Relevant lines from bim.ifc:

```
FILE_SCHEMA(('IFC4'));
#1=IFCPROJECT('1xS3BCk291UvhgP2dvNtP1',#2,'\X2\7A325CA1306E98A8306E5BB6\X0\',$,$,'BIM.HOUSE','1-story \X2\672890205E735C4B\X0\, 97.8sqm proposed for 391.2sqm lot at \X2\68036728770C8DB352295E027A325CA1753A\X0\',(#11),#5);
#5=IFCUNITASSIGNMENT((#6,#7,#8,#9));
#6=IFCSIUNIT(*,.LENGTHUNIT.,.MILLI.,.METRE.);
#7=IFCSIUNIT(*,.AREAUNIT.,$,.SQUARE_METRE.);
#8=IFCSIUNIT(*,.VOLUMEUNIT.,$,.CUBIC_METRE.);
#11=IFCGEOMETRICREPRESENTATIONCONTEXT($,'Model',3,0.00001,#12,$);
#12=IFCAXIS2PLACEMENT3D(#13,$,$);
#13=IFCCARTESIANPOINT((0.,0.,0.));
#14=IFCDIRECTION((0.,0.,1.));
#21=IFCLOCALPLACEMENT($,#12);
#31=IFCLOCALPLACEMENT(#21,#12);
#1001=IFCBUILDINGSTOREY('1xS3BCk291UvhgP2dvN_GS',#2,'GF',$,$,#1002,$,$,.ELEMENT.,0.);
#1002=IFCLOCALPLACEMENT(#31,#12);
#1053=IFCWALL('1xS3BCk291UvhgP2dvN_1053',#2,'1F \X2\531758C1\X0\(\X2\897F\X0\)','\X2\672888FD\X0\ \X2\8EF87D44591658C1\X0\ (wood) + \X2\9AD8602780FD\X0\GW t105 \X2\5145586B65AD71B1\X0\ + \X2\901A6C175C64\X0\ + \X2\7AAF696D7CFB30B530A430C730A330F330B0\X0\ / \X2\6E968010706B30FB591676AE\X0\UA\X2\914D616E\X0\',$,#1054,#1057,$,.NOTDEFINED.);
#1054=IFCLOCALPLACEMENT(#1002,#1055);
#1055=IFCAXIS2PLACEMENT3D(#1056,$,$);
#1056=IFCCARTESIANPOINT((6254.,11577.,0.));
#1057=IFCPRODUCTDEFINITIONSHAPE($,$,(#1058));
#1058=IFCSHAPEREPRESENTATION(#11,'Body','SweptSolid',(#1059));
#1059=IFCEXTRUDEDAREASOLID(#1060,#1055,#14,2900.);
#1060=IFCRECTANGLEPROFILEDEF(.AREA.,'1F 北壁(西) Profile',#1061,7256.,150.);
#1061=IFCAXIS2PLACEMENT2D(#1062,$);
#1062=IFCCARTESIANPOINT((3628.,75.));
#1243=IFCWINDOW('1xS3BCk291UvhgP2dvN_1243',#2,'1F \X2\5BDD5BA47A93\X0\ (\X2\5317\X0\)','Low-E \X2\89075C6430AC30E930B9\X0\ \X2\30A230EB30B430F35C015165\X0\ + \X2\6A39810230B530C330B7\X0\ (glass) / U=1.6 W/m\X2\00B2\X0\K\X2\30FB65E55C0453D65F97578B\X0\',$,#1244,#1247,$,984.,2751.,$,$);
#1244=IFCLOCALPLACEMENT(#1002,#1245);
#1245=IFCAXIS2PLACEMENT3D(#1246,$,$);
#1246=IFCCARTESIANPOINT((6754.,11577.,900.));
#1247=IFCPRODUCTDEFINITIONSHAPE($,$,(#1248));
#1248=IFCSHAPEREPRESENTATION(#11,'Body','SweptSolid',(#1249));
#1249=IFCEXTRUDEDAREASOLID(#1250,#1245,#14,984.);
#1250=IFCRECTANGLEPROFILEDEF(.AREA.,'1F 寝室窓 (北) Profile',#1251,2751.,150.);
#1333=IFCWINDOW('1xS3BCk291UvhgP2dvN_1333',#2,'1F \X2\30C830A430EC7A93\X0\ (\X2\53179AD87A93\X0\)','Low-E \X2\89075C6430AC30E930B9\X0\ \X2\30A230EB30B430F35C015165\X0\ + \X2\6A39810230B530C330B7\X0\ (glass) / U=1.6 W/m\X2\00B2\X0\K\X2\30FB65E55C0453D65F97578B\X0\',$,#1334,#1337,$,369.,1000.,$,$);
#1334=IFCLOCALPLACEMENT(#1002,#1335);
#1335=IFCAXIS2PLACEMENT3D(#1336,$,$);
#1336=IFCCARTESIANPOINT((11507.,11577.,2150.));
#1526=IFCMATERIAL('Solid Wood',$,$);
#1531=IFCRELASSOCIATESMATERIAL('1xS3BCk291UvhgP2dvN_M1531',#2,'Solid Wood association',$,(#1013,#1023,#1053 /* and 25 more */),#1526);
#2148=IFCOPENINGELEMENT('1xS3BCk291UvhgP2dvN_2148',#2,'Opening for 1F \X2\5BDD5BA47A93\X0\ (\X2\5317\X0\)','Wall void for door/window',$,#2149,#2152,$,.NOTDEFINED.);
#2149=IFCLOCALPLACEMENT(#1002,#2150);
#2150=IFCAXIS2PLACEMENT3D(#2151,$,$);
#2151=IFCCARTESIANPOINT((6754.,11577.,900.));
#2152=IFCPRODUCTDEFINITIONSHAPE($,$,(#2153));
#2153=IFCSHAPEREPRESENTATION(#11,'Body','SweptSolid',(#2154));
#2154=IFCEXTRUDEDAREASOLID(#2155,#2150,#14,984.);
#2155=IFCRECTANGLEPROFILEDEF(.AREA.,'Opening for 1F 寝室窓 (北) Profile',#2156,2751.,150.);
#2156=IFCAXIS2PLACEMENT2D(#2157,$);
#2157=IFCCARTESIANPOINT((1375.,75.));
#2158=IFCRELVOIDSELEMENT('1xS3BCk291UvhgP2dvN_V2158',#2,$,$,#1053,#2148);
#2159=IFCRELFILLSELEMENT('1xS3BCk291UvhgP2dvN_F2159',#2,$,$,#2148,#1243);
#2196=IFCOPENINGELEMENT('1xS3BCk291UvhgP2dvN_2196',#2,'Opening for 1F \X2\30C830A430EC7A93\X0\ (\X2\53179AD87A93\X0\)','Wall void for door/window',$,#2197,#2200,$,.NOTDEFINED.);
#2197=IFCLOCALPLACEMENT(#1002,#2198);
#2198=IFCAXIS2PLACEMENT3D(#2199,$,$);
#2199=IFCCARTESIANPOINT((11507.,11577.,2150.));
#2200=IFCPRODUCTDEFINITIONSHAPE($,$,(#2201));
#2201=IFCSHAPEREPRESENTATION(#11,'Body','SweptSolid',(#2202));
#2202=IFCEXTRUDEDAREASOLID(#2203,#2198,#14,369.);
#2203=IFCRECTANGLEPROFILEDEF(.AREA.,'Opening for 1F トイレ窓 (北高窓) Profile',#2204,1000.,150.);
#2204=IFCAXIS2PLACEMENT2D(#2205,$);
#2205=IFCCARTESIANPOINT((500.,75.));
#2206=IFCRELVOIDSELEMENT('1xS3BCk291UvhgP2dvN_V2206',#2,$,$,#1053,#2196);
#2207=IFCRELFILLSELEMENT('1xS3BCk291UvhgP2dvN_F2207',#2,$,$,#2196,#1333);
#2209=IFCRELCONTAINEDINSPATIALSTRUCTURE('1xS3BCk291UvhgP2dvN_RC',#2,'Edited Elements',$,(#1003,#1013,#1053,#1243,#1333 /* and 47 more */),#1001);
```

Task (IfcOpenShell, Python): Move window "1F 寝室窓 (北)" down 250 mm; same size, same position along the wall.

```python
import numpy as np
import ifcopenshell
import ifcopenshell.api.geometry
import ifcopenshell.util.placement
import ifcopenshell.util.unit

model = ifcopenshell.open("bim.ifc")
unit_scale = ifcopenshell.util.unit.calculate_unit_scale(model)

window = model.by_guid("1xS3BCk291UvhgP2dvN_1243")
opening = window.FillsVoids[0].RelatingOpeningElement
dz = -0.25 / unit_scale

shift = np.array([0.0, 0.0, dz])
# The window is not placed relative to its opening, so move both.
for product in (opening, window):
    matrix = ifcopenshell.util.placement.get_local_placement(product.ObjectPlacement)
    matrix[:3, 3] += shift
    ifcopenshell.api.geometry.edit_object_placement(model, product=product, matrix=matrix, is_si=False)

print(f"moved by {dz * unit_scale:+.3f} m")

model.write("bim_rev.ifc")
```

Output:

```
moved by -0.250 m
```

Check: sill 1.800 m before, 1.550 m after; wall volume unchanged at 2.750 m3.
